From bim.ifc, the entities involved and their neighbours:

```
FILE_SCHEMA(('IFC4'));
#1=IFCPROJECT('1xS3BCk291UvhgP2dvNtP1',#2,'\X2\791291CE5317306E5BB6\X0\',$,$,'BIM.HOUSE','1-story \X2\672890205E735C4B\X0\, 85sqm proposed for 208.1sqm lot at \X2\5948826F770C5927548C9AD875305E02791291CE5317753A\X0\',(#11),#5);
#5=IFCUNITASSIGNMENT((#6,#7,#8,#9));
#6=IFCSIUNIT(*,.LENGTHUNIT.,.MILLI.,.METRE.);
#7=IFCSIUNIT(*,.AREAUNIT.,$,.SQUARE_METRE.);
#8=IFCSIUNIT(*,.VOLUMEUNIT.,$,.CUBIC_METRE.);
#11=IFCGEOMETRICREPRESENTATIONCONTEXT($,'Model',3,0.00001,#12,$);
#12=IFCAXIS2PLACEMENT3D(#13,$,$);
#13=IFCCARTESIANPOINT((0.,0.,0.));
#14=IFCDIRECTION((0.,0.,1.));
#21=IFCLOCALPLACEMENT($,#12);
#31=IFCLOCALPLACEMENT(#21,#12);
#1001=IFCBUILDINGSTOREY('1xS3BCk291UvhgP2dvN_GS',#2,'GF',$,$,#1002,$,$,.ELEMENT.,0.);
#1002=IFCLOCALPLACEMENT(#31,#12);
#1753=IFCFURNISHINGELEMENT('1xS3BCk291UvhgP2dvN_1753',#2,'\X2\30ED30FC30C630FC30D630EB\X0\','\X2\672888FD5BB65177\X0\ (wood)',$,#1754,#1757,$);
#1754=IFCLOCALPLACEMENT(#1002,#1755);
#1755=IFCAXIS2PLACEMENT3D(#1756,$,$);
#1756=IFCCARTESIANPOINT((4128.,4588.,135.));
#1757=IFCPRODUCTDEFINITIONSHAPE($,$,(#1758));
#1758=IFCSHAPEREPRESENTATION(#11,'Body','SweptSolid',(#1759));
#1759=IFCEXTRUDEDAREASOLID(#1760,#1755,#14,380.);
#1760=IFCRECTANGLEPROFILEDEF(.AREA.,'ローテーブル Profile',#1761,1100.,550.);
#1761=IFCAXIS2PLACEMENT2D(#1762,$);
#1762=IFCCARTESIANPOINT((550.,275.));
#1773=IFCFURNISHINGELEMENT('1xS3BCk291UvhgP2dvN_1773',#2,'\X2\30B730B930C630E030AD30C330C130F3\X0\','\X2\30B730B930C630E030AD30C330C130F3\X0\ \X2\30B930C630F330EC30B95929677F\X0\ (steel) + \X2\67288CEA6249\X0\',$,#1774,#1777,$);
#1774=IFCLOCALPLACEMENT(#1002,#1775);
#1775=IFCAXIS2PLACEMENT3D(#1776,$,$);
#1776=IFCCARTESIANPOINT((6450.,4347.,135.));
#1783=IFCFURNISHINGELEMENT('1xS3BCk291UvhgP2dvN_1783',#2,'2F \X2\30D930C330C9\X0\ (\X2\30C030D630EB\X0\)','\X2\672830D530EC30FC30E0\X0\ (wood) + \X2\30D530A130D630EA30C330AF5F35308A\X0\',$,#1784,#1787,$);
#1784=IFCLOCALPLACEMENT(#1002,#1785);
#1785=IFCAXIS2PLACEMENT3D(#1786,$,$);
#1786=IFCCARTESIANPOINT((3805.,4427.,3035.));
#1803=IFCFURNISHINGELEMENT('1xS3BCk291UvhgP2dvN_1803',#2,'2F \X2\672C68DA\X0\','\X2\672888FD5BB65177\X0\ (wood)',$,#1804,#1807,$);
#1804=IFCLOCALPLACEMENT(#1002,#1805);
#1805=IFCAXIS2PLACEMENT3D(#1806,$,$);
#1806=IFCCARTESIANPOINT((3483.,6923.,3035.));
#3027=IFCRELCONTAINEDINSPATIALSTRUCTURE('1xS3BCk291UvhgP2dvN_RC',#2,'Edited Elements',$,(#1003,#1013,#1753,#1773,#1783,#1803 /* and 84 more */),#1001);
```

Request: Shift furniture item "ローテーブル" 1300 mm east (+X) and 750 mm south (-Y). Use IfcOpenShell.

```python
import ifcopenshell
import ifcopenshell.api.geometry
import ifcopenshell.util.placement

model = ifcopenshell.open("bim.ifc")

item = model.by_guid("1xS3BCk291UvhgP2dvN_1753")
matrix = ifcopenshell.util.placement.get_local_placement(item.ObjectPlacement)
matrix[0, 3] += 1300.0
matrix[1, 3] -= 750.0
ifcopenshell.api.geometry.edit_object_placement(model, product=item, matrix=matrix, is_si=False)

print(ifcopenshell.util.placement.get_local_placement(item.ObjectPlacement).round(3) + 0.0)

model.write("bim_rev.ifc")
```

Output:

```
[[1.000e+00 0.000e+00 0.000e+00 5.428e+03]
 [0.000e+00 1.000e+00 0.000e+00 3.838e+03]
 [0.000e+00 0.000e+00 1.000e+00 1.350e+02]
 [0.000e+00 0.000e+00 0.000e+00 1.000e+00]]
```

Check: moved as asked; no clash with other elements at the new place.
